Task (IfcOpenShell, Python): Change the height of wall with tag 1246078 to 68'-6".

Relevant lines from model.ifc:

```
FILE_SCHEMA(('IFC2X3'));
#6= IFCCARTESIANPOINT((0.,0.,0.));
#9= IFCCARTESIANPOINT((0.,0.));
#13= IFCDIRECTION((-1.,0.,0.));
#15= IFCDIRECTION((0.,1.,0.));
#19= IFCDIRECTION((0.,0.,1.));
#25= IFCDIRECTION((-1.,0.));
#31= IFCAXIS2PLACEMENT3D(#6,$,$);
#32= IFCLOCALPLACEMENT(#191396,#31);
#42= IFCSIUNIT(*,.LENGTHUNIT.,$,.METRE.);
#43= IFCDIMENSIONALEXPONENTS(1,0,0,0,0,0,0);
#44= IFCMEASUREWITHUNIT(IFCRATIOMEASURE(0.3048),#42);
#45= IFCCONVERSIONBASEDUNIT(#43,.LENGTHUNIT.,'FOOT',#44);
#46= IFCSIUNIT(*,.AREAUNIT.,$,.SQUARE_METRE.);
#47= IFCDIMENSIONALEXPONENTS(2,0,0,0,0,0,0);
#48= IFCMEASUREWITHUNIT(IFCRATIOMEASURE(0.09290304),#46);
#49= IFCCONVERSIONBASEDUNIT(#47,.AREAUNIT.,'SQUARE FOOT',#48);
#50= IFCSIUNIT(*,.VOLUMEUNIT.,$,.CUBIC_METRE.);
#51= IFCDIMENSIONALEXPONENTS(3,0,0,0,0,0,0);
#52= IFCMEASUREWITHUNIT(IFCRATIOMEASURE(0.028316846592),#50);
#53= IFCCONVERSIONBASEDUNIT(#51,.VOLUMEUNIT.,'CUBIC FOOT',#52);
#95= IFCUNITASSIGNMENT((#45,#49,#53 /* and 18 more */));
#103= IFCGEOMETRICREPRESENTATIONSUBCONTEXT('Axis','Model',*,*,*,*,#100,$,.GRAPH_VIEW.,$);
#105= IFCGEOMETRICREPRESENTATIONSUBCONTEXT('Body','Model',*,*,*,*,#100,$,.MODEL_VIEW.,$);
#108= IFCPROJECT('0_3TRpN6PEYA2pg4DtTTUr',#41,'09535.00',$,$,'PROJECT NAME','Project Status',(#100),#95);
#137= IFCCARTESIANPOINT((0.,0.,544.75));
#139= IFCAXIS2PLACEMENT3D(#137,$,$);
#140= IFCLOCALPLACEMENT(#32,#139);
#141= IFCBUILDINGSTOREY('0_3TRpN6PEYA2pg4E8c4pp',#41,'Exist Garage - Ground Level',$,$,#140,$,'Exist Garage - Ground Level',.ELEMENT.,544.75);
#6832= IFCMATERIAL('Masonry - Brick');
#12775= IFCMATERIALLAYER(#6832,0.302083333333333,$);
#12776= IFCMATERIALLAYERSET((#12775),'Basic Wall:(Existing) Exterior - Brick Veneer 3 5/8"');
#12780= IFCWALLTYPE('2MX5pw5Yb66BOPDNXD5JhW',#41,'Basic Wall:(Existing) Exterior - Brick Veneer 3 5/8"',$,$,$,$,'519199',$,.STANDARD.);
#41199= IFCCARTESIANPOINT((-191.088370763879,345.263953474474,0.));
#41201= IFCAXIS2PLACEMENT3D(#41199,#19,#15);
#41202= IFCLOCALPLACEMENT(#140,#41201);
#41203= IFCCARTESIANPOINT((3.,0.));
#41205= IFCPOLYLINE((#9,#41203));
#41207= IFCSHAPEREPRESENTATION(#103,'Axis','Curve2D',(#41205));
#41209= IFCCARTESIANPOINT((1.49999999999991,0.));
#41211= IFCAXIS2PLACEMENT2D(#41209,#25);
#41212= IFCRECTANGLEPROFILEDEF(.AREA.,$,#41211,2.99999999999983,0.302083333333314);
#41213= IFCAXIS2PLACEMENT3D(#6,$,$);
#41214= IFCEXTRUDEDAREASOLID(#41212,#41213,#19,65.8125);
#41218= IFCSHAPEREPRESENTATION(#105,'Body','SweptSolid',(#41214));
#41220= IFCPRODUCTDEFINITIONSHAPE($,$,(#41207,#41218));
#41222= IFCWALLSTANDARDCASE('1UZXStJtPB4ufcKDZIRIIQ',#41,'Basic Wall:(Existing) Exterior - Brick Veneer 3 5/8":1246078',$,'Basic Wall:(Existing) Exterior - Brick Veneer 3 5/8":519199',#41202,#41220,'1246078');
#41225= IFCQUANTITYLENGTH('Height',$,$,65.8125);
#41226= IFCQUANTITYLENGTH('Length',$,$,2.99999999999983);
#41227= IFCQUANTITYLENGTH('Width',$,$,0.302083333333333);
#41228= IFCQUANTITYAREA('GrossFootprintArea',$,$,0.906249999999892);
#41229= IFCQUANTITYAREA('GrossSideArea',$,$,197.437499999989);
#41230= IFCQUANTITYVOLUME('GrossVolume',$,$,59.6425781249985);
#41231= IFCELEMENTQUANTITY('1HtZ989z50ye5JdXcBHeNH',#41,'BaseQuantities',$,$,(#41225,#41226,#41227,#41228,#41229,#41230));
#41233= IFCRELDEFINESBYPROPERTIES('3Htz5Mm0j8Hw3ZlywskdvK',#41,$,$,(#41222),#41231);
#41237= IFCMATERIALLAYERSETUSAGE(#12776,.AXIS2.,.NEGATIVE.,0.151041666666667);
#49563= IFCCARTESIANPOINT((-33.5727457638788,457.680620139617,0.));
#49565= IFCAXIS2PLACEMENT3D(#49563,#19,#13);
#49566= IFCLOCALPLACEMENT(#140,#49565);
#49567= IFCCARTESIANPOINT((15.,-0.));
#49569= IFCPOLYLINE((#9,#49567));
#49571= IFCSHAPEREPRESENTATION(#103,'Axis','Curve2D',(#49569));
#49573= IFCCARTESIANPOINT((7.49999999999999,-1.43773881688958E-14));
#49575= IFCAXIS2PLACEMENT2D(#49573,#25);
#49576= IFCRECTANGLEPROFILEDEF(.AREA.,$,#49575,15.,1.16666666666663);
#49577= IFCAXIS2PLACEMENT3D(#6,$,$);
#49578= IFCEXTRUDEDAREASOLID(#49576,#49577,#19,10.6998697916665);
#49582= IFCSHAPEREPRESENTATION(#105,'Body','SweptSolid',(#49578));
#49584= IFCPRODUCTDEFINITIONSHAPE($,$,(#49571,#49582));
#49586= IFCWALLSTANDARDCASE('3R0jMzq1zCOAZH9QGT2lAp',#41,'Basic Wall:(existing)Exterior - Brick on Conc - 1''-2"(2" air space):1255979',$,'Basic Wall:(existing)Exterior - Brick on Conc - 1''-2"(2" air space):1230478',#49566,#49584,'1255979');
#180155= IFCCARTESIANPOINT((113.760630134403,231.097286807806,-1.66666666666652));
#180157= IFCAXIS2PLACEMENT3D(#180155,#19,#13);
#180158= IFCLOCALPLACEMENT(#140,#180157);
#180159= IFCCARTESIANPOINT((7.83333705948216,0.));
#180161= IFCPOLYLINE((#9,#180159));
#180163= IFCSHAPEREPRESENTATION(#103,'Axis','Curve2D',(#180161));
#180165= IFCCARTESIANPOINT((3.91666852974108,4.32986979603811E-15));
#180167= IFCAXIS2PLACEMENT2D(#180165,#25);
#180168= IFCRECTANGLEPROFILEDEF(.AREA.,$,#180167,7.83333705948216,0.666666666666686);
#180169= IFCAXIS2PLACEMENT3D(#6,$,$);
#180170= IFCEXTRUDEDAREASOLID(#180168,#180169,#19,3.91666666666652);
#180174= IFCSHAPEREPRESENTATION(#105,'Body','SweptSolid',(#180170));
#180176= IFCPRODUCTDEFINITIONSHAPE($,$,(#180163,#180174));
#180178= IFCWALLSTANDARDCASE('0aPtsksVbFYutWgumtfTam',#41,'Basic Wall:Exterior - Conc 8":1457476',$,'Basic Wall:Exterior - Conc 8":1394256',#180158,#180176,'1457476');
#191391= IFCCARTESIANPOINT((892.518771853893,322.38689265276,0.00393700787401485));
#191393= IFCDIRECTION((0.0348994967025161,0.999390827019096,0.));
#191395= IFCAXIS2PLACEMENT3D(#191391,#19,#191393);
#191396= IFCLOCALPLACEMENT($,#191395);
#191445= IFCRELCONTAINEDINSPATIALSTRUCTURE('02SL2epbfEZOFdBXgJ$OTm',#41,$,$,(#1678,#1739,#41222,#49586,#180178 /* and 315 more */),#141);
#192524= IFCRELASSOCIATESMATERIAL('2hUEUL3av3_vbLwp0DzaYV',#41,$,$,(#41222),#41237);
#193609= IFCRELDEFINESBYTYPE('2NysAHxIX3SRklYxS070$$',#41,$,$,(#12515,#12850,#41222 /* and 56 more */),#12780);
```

```python
import ifcopenshell
import ifcopenshell.api.pset
import ifcopenshell.geom
import ifcopenshell.util.element
import ifcopenshell.util.representation
import ifcopenshell.util.shape
import ifcopenshell.util.unit

model = ifcopenshell.open("model.ifc")
unit_scale = ifcopenshell.util.unit.calculate_unit_scale(model)
area_scale = ifcopenshell.util.unit.calculate_unit_scale(model, "AREAUNIT")
volume_scale = ifcopenshell.util.unit.calculate_unit_scale(model, "VOLUMEUNIT")
settings = ifcopenshell.geom.settings()


def volume(element):
    """Net volume in cubic metres, openings subtracted."""
    shape = ifcopenshell.geom.create_shape(settings, element)
    return ifcopenshell.util.shape.get_volume(shape.geometry)


wall = model.by_guid("1UZXStJtPB4ufcKDZIRIIQ")
before = volume(wall)

body = ifcopenshell.util.representation.get_representation(wall, "Model", "Body")
solid = body.Items[0]
old_height = solid.Depth
solid.Depth = 822 * 0.0254 / unit_scale
after = volume(wall)

# Update the stored height, areas and volumes.
qto = model.by_id(ifcopenshell.util.element.get_pset(wall, "BaseQuantities", should_inherit=False)["id"])
ifcopenshell.api.pset.edit_qto(model, qto=qto, properties={
    "Height": solid.Depth,
    "GrossSideArea": ifcopenshell.util.element.get_pset(wall, "BaseQuantities", "GrossSideArea") * solid.Depth / old_height,
    "GrossVolume": ifcopenshell.util.element.get_pset(wall, "BaseQuantities", "GrossVolume") * solid.Depth / old_height,
})

print(f"height {old_height:g} -> {solid.Depth:g}, volume {before:.3f} -> {after:.3f} m3")

model.write("model_rev.ifc")
```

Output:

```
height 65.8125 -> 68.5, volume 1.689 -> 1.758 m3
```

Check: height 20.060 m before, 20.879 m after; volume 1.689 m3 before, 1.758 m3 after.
